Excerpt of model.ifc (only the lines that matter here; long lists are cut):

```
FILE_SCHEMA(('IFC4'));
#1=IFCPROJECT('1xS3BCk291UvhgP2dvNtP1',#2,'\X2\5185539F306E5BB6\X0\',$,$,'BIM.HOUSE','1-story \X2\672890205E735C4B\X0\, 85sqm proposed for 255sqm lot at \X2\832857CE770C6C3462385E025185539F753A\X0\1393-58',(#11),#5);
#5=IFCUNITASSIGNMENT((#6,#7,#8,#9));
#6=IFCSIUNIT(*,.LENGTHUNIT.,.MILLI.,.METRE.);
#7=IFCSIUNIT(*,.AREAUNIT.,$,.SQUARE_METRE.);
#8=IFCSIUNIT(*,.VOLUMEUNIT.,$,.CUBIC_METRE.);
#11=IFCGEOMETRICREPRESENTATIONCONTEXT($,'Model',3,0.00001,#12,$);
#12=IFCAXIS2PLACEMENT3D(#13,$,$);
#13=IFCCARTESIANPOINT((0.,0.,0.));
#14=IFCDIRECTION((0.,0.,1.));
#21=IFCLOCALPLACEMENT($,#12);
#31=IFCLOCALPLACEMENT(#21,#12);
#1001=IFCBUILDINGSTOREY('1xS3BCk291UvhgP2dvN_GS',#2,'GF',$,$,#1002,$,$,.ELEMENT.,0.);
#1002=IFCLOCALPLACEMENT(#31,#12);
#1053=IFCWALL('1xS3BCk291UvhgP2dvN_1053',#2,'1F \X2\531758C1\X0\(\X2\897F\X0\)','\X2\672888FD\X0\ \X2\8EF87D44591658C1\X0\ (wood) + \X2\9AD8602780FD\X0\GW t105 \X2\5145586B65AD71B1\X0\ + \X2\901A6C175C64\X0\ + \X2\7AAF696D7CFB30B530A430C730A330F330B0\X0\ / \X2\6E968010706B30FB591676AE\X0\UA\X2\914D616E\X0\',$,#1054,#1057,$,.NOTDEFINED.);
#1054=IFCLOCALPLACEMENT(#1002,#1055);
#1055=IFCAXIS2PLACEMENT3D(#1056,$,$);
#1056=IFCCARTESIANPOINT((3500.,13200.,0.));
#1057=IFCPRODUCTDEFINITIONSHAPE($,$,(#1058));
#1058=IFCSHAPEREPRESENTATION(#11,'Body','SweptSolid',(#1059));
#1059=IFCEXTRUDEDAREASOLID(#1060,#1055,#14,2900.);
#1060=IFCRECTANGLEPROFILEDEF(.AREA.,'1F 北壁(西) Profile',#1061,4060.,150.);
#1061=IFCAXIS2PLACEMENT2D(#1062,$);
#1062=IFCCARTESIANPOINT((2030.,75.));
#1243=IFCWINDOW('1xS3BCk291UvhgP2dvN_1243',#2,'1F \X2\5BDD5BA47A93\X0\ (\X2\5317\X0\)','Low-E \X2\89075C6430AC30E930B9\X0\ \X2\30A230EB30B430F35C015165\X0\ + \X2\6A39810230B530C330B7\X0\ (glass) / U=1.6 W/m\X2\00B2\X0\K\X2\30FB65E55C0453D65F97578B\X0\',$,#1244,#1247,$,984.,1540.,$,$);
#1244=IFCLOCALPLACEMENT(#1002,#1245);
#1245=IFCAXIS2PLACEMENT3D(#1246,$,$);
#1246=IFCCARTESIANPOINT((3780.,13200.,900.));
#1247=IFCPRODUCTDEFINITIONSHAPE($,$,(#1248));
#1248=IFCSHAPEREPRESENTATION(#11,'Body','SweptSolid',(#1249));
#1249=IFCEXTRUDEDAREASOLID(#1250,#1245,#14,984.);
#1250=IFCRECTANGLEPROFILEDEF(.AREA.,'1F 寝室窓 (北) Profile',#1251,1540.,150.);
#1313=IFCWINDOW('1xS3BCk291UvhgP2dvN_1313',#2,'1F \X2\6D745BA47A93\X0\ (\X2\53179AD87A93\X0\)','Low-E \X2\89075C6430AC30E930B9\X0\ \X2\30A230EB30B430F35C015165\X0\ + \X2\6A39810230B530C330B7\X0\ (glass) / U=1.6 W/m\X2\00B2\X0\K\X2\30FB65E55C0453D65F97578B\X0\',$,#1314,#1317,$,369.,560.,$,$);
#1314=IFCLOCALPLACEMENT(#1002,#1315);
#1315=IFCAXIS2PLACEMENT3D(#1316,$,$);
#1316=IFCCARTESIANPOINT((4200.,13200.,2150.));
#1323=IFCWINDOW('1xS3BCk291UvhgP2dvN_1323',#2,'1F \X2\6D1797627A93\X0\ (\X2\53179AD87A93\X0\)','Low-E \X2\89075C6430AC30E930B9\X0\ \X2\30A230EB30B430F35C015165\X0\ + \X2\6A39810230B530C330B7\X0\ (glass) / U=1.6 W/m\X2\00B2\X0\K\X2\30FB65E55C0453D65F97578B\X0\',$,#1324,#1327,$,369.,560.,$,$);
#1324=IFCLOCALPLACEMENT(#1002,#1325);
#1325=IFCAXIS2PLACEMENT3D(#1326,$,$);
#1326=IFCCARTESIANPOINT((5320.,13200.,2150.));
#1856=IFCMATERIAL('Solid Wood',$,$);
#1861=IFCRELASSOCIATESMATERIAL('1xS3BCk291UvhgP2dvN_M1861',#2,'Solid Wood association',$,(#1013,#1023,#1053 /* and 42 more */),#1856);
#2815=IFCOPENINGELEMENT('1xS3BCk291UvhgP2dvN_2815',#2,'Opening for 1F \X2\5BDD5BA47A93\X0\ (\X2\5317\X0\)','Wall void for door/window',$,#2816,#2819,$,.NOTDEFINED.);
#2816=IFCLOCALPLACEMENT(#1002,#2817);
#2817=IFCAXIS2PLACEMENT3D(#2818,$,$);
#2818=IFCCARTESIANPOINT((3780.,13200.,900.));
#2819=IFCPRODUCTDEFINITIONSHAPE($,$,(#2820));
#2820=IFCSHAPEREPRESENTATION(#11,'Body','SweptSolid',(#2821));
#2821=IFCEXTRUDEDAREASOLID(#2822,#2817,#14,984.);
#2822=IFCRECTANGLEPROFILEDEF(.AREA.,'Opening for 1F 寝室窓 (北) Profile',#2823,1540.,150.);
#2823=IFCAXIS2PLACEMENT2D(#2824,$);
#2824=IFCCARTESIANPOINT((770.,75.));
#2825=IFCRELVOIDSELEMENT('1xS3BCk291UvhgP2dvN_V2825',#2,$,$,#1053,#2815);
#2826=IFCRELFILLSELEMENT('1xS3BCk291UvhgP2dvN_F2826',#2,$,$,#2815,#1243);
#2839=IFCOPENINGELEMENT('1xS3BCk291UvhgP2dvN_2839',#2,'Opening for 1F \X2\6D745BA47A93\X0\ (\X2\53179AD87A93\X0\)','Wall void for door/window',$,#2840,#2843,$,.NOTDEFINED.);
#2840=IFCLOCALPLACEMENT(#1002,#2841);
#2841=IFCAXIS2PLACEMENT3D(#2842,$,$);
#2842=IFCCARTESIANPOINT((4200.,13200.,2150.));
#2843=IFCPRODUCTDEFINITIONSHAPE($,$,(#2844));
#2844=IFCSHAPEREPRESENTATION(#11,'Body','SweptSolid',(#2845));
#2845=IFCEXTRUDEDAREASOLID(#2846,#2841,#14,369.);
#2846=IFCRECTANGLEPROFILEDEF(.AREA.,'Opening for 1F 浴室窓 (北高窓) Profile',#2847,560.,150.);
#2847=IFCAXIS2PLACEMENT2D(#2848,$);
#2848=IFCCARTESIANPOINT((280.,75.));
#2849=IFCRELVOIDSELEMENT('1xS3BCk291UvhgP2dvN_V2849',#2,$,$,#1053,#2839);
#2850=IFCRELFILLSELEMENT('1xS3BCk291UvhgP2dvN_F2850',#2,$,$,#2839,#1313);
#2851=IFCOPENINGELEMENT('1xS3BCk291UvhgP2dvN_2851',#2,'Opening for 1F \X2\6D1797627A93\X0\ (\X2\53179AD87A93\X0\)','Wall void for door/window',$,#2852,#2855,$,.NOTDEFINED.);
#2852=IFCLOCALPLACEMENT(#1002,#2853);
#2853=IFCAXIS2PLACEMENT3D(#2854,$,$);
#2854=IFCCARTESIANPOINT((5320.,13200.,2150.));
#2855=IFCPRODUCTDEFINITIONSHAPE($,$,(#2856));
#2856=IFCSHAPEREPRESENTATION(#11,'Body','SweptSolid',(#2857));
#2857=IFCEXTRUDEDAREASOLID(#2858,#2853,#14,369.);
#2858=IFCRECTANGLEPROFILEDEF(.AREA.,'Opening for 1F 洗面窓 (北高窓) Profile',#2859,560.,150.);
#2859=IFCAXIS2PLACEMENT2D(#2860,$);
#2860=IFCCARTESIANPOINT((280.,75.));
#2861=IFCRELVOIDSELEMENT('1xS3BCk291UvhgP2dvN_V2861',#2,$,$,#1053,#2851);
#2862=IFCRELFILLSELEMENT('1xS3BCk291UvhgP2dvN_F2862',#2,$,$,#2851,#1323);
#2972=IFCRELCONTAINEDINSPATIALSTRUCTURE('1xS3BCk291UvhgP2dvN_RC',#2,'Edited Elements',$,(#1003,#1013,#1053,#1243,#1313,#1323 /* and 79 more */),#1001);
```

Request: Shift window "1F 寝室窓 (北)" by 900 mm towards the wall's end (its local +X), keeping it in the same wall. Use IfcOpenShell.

```python
import ifcopenshell
import ifcopenshell.api.geometry
import ifcopenshell.util.placement
import ifcopenshell.util.unit

model = ifcopenshell.open("model.ifc")
unit_scale = ifcopenshell.util.unit.calculate_unit_scale(model)

window = model.by_id(1243)
opening = window.FillsVoids[0].RelatingOpeningElement
wall = opening.VoidsElements[0].RelatingBuildingElement

wall_matrix = ifcopenshell.util.placement.get_local_placement(wall.ObjectPlacement)
shift = wall_matrix[:3, 0] * 0.9 / unit_scale
before = ifcopenshell.util.placement.get_local_placement(window.ObjectPlacement)[:3, 3].copy()

# The window is not placed relative to its opening, so move both.
for product in (opening, window):
    matrix = ifcopenshell.util.placement.get_local_placement(product.ObjectPlacement)
    matrix[:3, 3] += shift
    ifcopenshell.api.geometry.edit_object_placement(model, product=product, matrix=matrix, is_si=False)

after = ifcopenshell.util.placement.get_local_placement(window.ObjectPlacement)[:3, 3]
print("window moved by", (after - before).round(3) + 0.0)

model.write("model_v2.ifc")
```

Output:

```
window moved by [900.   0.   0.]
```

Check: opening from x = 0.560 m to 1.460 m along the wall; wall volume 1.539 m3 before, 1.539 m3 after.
